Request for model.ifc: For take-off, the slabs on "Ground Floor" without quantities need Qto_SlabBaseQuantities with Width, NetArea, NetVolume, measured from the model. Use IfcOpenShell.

First a look at what the model holds.

```python
import ifcopenshell
import ifcopenshell.util.element
import ifcopenshell.util.unit

model = ifcopenshell.open("model.ifc")
print(model.schema)
for unit_type in ("LENGTHUNIT", "AREAUNIT", "VOLUMEUNIT"):
    print(unit_type, ifcopenshell.util.unit.calculate_unit_scale(model, unit_type))
storey = next(s for s in model.by_type("IfcBuildingStorey") if s.Name == "Ground Floor")
slabs = [e for e in ifcopenshell.util.element.get_decomposition(storey) if e.is_a("IfcSlab")]
for e in sorted(slabs, key=lambda e: e.id()):
    print(e.id(), e.is_a(), e.Name, list(ifcopenshell.util.element.get_psets(e, qtos_only=True)), sep=" | ")
```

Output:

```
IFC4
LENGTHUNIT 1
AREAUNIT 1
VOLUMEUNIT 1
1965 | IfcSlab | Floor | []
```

```python
import ifcopenshell
import ifcopenshell.api.pset
import ifcopenshell.geom
import ifcopenshell.util.element
import ifcopenshell.util.shape
import ifcopenshell.util.unit

model = ifcopenshell.open("model.ifc")
unit_scale = ifcopenshell.util.unit.calculate_unit_scale(model)
area_scale = ifcopenshell.util.unit.calculate_unit_scale(model, "AREAUNIT")
volume_scale = ifcopenshell.util.unit.calculate_unit_scale(model, "VOLUMEUNIT")
settings = ifcopenshell.geom.settings()

storey = next(s for s in model.by_type("IfcBuildingStorey") if s.Name == "Ground Floor")
slabs = [e for e in ifcopenshell.util.element.get_decomposition(storey) if e.is_a("IfcSlab")]

for e in sorted(slabs, key=lambda e: e.id()):
    if ifcopenshell.util.element.get_psets(e, qtos_only=True, should_inherit=False):
        continue
    # Geometry comes back in metres, in the element's own axes.
    shape = ifcopenshell.geom.create_shape(settings, e)
    values = {
        "Width": ifcopenshell.util.shape.get_z(shape.geometry) / unit_scale,
        "NetArea": ifcopenshell.util.shape.get_footprint_area(shape.geometry) / area_scale,
        "NetVolume": ifcopenshell.util.shape.get_volume(shape.geometry) / volume_scale,
    }
    qto = ifcopenshell.api.pset.add_qto(model, product=e, name="Qto_SlabBaseQuantities")
    ifcopenshell.api.pset.edit_qto(model, qto=qto, properties=values)
    print(e.id(), {k: round(v, 3) for k, v in values.items()})

model.write("model_v2.ifc")
```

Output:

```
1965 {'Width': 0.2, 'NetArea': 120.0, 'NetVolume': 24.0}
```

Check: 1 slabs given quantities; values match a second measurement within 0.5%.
